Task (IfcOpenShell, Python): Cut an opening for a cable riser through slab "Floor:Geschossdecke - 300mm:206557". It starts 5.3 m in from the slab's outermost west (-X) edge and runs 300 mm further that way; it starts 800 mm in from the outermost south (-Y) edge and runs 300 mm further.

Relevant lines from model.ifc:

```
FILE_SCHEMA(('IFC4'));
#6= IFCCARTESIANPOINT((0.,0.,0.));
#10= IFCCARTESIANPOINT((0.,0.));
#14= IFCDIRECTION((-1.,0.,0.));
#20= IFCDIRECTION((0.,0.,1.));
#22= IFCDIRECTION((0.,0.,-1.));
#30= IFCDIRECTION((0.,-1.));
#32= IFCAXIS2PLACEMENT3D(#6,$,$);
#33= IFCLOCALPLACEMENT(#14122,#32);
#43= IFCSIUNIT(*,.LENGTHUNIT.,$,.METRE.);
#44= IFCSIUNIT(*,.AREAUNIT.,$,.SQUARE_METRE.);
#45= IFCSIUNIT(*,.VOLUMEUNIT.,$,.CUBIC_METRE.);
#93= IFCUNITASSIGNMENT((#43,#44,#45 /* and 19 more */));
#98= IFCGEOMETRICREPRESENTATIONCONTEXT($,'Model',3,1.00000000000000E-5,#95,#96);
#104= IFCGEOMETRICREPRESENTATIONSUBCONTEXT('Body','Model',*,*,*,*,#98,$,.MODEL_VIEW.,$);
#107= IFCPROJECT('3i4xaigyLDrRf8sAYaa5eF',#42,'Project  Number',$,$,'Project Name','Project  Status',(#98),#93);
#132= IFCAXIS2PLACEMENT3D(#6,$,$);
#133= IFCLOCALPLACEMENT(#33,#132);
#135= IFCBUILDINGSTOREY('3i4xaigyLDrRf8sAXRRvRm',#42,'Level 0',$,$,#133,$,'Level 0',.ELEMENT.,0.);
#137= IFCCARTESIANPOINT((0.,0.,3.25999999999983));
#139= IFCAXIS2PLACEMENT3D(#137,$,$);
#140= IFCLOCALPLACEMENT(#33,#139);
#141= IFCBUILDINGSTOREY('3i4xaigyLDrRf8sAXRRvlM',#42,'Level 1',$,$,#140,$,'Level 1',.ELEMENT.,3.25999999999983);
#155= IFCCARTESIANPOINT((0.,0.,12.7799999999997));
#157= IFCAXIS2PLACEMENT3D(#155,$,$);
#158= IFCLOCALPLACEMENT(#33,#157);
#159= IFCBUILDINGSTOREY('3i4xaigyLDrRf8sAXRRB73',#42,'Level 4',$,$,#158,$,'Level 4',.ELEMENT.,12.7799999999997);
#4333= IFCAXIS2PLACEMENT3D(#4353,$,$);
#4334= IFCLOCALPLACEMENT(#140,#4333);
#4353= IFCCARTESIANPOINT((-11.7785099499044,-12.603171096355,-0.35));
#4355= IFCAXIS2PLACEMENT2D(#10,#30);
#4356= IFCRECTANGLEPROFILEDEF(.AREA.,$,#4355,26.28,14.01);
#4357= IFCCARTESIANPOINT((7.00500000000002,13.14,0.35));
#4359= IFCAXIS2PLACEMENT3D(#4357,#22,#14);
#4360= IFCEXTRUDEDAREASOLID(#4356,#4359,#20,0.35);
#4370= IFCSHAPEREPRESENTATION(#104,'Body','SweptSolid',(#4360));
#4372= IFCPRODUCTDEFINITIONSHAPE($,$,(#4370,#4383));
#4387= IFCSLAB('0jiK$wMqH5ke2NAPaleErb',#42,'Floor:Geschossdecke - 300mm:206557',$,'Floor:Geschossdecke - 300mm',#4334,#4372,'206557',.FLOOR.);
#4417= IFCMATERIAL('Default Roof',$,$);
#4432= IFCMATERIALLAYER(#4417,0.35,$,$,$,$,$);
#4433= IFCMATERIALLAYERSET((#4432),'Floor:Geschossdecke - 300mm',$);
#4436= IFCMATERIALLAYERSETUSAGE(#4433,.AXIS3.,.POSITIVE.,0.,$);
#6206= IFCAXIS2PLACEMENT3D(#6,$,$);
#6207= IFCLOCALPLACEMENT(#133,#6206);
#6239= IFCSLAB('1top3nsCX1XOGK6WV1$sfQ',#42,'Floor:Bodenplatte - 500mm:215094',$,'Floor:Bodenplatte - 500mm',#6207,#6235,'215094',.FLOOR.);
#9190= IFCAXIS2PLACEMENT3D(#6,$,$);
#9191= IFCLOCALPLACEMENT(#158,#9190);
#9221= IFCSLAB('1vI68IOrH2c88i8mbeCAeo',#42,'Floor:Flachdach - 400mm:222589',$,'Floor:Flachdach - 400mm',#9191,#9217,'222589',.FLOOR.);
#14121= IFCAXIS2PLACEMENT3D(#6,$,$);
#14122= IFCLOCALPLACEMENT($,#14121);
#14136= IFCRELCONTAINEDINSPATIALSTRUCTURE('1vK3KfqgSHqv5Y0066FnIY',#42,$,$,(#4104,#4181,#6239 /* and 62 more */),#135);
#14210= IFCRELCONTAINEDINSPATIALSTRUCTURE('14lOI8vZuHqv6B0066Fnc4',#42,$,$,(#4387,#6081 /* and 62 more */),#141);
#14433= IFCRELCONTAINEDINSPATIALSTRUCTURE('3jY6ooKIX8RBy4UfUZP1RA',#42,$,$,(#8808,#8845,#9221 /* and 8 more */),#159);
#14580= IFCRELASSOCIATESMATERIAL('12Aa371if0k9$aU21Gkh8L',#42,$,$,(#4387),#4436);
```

```python
import numpy as np
import ifcopenshell
import ifcopenshell.api.feature
import ifcopenshell.api.geometry
import ifcopenshell.api.root
import ifcopenshell.geom
import ifcopenshell.util.placement
import ifcopenshell.util.representation
import ifcopenshell.util.shape
import ifcopenshell.util.unit

model = ifcopenshell.open("model.ifc")
unit_scale = ifcopenshell.util.unit.calculate_unit_scale(model)
settings = ifcopenshell.geom.settings()


def volume(element):
    """Net volume in cubic metres, openings subtracted."""
    shape = ifcopenshell.geom.create_shape(settings, element)
    return ifcopenshell.util.shape.get_volume(shape.geometry)


slab = model.by_guid("0jiK$wMqH5ke2NAPaleErb")
before = volume(slab)

# Extent in the slab's own axes, in metres. The edges named are its -X and -Y sides.
slab_shape = ifcopenshell.geom.create_shape(settings, slab)
vertices = ifcopenshell.util.shape.get_vertices(slab_shape.geometry)
x_min, y_min, bottom = vertices.min(axis=0)
top = vertices[:, 2].max()

opening = ifcopenshell.api.root.create_entity(model, ifc_class="IfcOpeningElement", name="Cable riser opening", predefined_type="OPENING")
context = ifcopenshell.util.representation.get_context(model, "Model", "Body", "MODEL_VIEW")
width, depth = 0.3, 0.3
outline = [(0.0, 0.0), (width, 0.0), (width, depth), (0.0, depth), (0.0, 0.0)]
# Overshoot both faces by 50 mm so the cut is clean.
shape = ifcopenshell.api.geometry.add_slab_representation(
    model, context=context, depth=top - bottom + 0.1, polyline=outline
)
ifcopenshell.api.geometry.assign_representation(model, product=opening, representation=shape)

matrix = ifcopenshell.util.placement.get_local_placement(slab.ObjectPlacement)
matrix[:, 3] = matrix @ np.append(np.array([x_min + 5.3, y_min + 0.8, bottom - 0.05]) / unit_scale, 1.0)
ifcopenshell.api.geometry.edit_object_placement(model, product=opening, matrix=matrix, is_si=False)
ifcopenshell.api.feature.add_feature(model, feature=opening, element=slab)

after = volume(slab)

print(f"slab volume {before:.3f} -> {after:.3f} m3")

model.write("model-out.ifc")
```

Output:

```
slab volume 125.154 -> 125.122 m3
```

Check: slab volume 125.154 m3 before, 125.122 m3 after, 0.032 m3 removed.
